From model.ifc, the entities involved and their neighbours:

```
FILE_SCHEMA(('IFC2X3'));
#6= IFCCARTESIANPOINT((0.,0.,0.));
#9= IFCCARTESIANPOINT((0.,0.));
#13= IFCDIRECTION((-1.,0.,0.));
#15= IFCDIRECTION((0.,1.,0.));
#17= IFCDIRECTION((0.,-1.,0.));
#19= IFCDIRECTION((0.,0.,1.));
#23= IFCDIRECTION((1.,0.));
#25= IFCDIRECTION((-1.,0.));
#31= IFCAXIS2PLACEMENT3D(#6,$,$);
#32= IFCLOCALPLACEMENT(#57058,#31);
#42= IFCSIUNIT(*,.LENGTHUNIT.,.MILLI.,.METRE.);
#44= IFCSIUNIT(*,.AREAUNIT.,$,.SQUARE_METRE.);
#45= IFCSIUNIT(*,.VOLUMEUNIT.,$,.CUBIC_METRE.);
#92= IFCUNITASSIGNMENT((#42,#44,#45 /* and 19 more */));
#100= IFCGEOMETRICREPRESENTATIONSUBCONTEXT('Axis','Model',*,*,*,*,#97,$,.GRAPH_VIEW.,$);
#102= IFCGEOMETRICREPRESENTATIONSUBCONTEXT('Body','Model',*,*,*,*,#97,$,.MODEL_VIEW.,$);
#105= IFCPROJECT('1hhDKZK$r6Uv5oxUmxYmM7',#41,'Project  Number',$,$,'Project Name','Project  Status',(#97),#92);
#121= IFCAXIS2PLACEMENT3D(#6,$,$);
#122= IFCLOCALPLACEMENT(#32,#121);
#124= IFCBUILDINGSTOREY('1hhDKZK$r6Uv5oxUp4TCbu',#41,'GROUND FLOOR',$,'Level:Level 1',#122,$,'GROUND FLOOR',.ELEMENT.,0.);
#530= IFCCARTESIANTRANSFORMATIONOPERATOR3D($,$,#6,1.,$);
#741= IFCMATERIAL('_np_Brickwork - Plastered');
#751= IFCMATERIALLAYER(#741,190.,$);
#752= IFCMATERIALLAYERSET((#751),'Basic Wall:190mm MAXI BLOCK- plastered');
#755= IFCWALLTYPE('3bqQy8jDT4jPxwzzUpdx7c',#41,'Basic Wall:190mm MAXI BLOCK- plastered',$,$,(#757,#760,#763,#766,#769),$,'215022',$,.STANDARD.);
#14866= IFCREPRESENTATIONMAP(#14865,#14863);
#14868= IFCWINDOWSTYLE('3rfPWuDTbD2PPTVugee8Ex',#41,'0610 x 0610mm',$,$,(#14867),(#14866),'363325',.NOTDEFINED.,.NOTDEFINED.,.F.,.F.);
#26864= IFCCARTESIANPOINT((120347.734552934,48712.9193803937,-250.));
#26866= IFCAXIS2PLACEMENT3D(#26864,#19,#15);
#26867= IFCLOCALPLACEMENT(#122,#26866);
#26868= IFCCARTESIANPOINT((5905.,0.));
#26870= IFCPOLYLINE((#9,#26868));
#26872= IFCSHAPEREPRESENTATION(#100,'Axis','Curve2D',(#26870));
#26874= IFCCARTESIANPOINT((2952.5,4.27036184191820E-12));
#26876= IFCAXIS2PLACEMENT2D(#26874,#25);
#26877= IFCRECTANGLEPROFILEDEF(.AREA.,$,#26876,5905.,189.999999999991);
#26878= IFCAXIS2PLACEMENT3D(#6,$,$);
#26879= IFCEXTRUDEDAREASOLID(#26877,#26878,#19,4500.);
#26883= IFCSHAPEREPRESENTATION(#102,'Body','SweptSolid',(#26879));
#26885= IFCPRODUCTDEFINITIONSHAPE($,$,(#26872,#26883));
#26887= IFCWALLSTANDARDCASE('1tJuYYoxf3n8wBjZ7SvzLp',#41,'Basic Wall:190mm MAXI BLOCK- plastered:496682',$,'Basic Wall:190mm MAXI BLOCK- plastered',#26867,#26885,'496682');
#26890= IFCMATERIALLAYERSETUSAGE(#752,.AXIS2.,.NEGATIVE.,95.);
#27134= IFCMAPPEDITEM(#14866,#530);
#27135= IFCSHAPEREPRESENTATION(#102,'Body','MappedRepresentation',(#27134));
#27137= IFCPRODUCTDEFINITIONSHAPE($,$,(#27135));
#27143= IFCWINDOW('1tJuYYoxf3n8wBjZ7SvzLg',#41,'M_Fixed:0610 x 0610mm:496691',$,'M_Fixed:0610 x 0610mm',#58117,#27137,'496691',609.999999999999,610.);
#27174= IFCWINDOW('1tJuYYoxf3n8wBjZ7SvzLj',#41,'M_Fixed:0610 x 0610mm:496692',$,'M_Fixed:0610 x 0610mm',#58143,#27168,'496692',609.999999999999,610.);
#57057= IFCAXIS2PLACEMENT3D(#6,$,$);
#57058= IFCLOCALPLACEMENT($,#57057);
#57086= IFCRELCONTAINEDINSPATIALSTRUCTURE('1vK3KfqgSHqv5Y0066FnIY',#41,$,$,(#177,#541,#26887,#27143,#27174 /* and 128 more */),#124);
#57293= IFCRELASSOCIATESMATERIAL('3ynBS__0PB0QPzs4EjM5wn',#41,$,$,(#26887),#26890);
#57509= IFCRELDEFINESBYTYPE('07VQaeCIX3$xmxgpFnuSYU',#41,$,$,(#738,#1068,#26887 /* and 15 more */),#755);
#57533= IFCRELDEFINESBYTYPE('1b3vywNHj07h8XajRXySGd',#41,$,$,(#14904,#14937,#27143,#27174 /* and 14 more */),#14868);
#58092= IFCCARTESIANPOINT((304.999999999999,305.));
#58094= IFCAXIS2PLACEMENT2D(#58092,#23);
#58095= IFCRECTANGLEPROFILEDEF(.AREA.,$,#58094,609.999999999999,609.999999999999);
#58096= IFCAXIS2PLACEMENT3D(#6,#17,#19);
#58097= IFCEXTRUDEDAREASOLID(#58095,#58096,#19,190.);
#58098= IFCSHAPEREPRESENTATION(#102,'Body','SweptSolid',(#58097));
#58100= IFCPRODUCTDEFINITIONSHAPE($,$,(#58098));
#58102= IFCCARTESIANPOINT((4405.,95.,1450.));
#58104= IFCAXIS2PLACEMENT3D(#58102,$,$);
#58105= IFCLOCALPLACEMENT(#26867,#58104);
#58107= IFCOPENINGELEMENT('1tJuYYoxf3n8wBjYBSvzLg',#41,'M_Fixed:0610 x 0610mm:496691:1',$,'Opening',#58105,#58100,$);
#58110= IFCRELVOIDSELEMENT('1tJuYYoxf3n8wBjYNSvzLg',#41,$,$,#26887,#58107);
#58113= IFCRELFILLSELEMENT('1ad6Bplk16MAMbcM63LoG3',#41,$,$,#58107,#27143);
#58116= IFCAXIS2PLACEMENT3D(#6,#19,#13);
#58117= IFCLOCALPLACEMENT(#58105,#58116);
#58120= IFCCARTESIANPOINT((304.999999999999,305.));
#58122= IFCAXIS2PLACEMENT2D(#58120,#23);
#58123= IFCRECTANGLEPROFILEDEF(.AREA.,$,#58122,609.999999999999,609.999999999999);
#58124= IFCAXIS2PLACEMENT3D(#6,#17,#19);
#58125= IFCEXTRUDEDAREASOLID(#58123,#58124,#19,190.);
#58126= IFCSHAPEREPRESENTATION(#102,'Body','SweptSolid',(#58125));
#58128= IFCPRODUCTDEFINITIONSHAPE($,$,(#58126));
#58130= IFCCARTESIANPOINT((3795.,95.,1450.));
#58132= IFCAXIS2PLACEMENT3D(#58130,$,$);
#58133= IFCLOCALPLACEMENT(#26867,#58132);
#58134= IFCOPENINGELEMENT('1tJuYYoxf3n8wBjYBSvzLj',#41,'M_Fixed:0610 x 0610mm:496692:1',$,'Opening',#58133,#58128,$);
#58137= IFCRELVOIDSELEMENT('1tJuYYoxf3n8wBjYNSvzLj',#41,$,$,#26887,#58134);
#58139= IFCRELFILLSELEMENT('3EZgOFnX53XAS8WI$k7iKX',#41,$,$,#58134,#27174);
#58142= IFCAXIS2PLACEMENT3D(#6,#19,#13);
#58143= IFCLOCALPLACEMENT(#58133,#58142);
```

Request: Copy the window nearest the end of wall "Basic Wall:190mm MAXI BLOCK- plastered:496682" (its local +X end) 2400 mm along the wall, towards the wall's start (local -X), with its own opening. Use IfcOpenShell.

```python
import ifcopenshell
import ifcopenshell.api.feature
import ifcopenshell.api.geometry
import ifcopenshell.api.root
import ifcopenshell.geom
import ifcopenshell.util.element
import ifcopenshell.util.placement
import ifcopenshell.util.shape
import ifcopenshell.util.unit

model = ifcopenshell.open("model.ifc")
unit_scale = ifcopenshell.util.unit.calculate_unit_scale(model)
settings = ifcopenshell.geom.settings()


def volume(element):
    """Net volume in cubic metres, openings subtracted."""
    shape = ifcopenshell.geom.create_shape(settings, element)
    return ifcopenshell.util.shape.get_volume(shape.geometry)


def reuse_history(source, copy):
    """copy_class also copies each property set's owner history, people and application; keep the originals."""
    for rel in copy.IsDefinedBy:
        if rel.is_a("IfcRelDefinesByProperties") and (history := rel.RelatingPropertyDefinition.OwnerHistory):
            rel.RelatingPropertyDefinition.OwnerHistory = source.OwnerHistory
            ifcopenshell.util.element.remove_deep2(model, history)


window = model.by_id(27143)
opening = window.FillsVoids[0].RelatingOpeningElement
wall = opening.VoidsElements[0].RelatingBuildingElement
before = volume(wall)
shift = ifcopenshell.util.placement.get_local_placement(wall.ObjectPlacement)[:3, 0] * -2.4 / unit_scale

# copy_class copies the void relationship, type, container and properties, but no geometry.
new_opening = ifcopenshell.api.root.copy_class(model, product=opening)
new_opening.Representation = ifcopenshell.util.element.copy_deep(
    model, opening.Representation, exclude=["IfcGeometricRepresentationContext", "IfcRepresentationMap"]
)
new_opening.Name = "M_Fixed:0610 x 0610mm"
new_window = ifcopenshell.api.root.copy_class(model, product=window)
new_window.Representation = ifcopenshell.util.element.copy_deep(
    model, window.Representation, exclude=["IfcGeometricRepresentationContext", "IfcRepresentationMap"]
)
new_window.Name = "M_Fixed:0610 x 0610mm"
new_window.Tag = None
reuse_history(window, new_window)
fills = ifcopenshell.api.feature.add_filling(model, opening=new_opening, element=new_window)
fills.OwnerHistory = new_window.OwnerHistory  # required in IFC2X3

for old, new in ((opening, new_opening), (window, new_window)):
    matrix = ifcopenshell.util.placement.get_local_placement(old.ObjectPlacement)
    matrix[:3, 3] += shift
    ifcopenshell.api.geometry.edit_object_placement(model, product=new, matrix=matrix, is_si=False)

after = volume(wall)

print(f"wall volume {before:.3f} -> {after:.3f} m3")

model.write("model_updated.ifc")
```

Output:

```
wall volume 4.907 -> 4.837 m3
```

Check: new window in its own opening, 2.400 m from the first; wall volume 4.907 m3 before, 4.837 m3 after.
